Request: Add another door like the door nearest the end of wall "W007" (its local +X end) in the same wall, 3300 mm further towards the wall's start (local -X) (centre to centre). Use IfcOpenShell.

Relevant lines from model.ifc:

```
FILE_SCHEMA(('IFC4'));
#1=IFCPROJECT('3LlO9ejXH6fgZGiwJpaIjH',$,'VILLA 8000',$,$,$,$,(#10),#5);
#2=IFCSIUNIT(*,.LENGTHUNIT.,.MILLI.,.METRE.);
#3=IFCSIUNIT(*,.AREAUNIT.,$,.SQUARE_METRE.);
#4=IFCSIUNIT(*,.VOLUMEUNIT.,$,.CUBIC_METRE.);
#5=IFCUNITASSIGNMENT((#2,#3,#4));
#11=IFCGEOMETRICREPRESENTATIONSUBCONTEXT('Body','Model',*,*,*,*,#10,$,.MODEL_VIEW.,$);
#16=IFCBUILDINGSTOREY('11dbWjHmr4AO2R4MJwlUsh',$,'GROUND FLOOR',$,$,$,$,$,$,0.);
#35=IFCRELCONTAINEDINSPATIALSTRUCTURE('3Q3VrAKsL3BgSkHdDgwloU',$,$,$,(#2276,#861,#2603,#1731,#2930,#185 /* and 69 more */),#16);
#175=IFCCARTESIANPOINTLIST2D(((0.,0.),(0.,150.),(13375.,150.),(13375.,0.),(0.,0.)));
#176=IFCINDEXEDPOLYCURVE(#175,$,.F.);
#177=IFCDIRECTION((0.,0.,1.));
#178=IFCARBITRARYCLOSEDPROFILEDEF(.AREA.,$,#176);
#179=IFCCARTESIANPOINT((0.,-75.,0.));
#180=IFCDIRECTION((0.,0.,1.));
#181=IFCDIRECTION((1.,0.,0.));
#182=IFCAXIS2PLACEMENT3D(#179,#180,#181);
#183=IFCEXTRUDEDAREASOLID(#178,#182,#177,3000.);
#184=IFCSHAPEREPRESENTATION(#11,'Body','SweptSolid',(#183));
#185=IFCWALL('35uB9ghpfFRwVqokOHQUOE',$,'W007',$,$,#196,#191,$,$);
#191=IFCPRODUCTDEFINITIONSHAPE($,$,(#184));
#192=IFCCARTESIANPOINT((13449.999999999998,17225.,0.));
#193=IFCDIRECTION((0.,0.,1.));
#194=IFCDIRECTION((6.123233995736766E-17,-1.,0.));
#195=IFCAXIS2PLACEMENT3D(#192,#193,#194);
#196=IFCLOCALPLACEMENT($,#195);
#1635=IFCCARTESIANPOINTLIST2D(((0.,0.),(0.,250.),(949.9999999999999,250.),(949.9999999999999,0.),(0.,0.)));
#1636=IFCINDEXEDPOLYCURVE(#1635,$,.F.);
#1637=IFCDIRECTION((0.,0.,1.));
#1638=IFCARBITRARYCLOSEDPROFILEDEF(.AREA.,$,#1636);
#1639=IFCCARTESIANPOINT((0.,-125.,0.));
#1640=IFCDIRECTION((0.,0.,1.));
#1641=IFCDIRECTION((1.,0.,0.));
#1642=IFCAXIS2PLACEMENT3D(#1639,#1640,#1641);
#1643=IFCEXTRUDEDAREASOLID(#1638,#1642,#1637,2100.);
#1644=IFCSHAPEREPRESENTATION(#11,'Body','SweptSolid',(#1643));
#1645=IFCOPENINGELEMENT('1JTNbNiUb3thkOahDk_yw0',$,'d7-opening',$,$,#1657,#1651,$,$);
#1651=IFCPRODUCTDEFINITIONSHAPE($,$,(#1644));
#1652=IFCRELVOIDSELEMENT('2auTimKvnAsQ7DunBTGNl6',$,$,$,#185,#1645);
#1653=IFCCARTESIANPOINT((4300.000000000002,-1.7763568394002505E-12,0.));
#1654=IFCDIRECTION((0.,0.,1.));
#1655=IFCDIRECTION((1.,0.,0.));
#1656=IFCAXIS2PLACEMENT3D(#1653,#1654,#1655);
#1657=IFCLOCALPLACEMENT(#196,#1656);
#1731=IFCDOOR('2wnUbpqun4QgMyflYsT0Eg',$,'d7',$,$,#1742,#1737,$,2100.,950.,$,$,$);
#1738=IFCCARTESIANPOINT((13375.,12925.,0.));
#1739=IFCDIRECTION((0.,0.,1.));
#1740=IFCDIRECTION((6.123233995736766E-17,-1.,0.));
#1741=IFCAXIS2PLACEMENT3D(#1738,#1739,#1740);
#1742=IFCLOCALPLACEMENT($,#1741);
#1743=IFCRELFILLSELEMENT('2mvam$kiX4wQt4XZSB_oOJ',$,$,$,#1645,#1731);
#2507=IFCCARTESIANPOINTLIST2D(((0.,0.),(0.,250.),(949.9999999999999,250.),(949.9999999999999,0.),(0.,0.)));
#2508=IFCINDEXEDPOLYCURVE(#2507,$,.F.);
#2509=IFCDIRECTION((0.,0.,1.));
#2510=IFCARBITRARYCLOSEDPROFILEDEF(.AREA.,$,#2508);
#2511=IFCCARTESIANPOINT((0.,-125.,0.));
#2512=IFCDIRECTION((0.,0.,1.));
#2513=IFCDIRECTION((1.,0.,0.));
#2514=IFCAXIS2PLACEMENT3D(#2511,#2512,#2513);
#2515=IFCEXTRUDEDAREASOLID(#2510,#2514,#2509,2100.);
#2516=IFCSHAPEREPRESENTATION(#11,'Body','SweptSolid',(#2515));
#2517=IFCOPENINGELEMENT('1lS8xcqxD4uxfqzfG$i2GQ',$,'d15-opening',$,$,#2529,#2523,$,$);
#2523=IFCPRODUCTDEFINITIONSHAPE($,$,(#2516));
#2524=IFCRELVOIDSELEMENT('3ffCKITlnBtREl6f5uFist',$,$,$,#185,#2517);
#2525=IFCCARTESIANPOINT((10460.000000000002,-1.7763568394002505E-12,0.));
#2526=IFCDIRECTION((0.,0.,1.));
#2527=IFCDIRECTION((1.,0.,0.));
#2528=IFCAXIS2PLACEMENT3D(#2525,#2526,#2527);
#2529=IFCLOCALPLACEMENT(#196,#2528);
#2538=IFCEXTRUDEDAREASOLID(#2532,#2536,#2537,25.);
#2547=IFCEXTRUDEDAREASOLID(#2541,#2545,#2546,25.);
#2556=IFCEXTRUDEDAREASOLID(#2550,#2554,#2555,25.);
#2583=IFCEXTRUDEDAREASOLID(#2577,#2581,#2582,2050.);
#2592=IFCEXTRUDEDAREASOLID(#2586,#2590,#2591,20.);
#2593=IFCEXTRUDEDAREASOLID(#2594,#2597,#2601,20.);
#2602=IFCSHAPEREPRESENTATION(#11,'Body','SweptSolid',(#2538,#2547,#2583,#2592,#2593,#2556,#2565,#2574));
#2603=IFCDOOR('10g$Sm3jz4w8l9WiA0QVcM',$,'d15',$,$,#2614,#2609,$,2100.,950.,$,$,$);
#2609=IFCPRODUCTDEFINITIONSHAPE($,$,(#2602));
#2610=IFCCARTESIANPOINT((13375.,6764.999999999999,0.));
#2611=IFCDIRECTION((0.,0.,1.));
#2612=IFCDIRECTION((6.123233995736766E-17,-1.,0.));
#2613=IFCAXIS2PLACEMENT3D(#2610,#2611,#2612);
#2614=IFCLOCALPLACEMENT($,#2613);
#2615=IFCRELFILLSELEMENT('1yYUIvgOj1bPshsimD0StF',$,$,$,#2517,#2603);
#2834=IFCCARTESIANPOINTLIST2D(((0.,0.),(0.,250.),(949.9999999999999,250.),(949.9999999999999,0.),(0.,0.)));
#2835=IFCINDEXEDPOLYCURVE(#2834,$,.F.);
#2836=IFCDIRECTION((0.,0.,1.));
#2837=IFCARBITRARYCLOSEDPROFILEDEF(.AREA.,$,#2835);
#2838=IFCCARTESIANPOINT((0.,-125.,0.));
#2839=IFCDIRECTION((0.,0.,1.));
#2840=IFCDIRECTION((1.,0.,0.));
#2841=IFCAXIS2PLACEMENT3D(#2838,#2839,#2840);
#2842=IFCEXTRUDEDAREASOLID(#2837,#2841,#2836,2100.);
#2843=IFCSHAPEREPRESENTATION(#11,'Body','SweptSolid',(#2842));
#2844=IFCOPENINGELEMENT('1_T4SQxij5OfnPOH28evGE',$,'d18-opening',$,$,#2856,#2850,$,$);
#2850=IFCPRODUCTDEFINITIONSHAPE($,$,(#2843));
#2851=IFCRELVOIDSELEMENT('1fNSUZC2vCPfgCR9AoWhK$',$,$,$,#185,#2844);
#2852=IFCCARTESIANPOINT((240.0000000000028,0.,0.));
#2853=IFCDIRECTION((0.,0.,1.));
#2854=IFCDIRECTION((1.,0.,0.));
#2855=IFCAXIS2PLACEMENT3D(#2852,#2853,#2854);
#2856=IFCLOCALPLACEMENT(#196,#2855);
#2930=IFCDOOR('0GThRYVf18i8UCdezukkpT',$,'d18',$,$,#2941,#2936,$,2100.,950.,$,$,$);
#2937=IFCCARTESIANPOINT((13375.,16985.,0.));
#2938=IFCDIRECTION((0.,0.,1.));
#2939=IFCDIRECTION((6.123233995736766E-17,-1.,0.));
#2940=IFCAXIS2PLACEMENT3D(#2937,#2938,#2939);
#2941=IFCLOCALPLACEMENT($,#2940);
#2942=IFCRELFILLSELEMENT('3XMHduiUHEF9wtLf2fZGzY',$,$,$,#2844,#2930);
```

```python
import ifcopenshell
import ifcopenshell.api.feature
import ifcopenshell.api.geometry
import ifcopenshell.api.root
import ifcopenshell.geom
import ifcopenshell.util.element
import ifcopenshell.util.placement
import ifcopenshell.util.shape
import ifcopenshell.util.unit

model = ifcopenshell.open("model.ifc")
unit_scale = ifcopenshell.util.unit.calculate_unit_scale(model)
settings = ifcopenshell.geom.settings()


def volume(element):
    """Net volume in cubic metres, openings subtracted."""
    shape = ifcopenshell.geom.create_shape(settings, element)
    return ifcopenshell.util.shape.get_volume(shape.geometry)


door = model.by_guid("10g$Sm3jz4w8l9WiA0QVcM")
opening = door.FillsVoids[0].RelatingOpeningElement
wall = opening.VoidsElements[0].RelatingBuildingElement
before = volume(wall)
shift = ifcopenshell.util.placement.get_local_placement(wall.ObjectPlacement)[:3, 0] * -3.3 / unit_scale

# copy_class copies the void relationship, type, container and properties, but no geometry.
new_opening = ifcopenshell.api.root.copy_class(model, product=opening)
new_opening.Representation = ifcopenshell.util.element.copy_deep(
    model, opening.Representation, exclude=["IfcGeometricRepresentationContext", "IfcRepresentationMap"]
)
new_door = ifcopenshell.api.root.copy_class(model, product=door)
new_door.Representation = ifcopenshell.util.element.copy_deep(
    model, door.Representation, exclude=["IfcGeometricRepresentationContext", "IfcRepresentationMap"]
)
ifcopenshell.api.feature.add_filling(model, opening=new_opening, element=new_door)

for old, new in ((opening, new_opening), (door, new_door)):
    matrix = ifcopenshell.util.placement.get_local_placement(old.ObjectPlacement)
    matrix[:3, 3] += shift
    ifcopenshell.api.geometry.edit_object_placement(model, product=new, matrix=matrix, is_si=False)

after = volume(wall)

print(f"wall volume {before:.3f} -> {after:.3f} m3")

model.write("model_updated.ifc")
```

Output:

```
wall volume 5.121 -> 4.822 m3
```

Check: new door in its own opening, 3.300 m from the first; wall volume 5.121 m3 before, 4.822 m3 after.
